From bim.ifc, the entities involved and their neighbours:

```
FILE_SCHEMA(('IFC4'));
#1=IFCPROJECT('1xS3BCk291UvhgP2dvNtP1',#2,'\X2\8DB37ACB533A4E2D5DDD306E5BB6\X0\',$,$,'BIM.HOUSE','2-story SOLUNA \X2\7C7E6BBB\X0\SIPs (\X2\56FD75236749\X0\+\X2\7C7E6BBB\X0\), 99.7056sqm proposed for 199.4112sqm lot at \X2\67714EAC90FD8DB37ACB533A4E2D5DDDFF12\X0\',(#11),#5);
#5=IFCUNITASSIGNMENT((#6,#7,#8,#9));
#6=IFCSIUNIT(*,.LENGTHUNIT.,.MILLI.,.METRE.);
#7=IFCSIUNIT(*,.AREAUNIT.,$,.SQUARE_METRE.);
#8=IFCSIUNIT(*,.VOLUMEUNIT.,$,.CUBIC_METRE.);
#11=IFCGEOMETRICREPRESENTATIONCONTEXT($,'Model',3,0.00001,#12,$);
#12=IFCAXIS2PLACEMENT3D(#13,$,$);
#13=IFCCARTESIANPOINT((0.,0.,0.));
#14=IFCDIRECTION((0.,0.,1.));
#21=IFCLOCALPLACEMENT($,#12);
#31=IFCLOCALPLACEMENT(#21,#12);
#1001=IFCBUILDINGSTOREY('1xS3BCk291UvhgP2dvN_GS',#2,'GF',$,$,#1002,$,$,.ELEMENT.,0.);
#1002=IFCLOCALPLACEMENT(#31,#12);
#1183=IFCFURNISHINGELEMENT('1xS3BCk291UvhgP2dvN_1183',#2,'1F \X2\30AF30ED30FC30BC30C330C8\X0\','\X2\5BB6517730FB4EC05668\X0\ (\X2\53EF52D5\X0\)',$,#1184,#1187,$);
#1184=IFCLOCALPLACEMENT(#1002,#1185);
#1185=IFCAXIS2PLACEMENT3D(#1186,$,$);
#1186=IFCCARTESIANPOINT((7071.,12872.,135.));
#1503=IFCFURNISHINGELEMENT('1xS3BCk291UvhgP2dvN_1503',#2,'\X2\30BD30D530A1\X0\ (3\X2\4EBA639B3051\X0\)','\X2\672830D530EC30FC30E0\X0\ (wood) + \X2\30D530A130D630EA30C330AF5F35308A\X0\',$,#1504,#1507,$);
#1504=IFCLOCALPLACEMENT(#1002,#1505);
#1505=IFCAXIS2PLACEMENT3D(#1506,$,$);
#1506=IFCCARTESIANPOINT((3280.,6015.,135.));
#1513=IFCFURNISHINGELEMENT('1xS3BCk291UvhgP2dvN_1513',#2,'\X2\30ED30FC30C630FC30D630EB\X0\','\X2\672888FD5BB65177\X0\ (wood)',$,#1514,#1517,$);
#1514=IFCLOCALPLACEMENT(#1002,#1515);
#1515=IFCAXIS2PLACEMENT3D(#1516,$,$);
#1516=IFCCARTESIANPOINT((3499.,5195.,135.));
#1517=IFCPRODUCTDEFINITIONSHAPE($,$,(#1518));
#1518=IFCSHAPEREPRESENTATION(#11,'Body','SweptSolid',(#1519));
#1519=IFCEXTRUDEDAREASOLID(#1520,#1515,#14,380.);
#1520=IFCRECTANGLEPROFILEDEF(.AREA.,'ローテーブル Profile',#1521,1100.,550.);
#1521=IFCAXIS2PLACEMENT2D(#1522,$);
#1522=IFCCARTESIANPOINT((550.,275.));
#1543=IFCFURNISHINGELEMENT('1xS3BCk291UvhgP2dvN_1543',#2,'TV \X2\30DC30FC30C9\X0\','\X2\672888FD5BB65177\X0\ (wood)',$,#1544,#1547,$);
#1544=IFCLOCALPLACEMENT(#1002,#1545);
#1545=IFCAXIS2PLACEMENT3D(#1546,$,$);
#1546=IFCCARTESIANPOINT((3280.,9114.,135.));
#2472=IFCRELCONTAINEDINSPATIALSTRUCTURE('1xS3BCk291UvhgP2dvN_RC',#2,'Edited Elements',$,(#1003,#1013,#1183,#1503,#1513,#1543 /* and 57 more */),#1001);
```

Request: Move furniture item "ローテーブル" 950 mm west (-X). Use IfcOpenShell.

```python
import ifcopenshell
import ifcopenshell.api.geometry
import ifcopenshell.util.placement
import ifcopenshell.util.unit

model = ifcopenshell.open("bim.ifc")
unit_scale = ifcopenshell.util.unit.calculate_unit_scale(model)

item = model.by_id(1513)
matrix = ifcopenshell.util.placement.get_local_placement(item.ObjectPlacement)
matrix[0, 3] -= 0.95 / unit_scale
ifcopenshell.api.geometry.edit_object_placement(model, product=item, matrix=matrix, is_si=False)

print(ifcopenshell.util.placement.get_local_placement(item.ObjectPlacement).round(3) + 0.0)

model.write("bim-out.ifc")
```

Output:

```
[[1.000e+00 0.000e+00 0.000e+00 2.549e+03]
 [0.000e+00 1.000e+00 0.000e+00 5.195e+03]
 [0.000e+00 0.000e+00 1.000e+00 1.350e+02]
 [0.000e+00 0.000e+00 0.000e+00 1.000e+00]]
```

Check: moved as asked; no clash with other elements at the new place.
